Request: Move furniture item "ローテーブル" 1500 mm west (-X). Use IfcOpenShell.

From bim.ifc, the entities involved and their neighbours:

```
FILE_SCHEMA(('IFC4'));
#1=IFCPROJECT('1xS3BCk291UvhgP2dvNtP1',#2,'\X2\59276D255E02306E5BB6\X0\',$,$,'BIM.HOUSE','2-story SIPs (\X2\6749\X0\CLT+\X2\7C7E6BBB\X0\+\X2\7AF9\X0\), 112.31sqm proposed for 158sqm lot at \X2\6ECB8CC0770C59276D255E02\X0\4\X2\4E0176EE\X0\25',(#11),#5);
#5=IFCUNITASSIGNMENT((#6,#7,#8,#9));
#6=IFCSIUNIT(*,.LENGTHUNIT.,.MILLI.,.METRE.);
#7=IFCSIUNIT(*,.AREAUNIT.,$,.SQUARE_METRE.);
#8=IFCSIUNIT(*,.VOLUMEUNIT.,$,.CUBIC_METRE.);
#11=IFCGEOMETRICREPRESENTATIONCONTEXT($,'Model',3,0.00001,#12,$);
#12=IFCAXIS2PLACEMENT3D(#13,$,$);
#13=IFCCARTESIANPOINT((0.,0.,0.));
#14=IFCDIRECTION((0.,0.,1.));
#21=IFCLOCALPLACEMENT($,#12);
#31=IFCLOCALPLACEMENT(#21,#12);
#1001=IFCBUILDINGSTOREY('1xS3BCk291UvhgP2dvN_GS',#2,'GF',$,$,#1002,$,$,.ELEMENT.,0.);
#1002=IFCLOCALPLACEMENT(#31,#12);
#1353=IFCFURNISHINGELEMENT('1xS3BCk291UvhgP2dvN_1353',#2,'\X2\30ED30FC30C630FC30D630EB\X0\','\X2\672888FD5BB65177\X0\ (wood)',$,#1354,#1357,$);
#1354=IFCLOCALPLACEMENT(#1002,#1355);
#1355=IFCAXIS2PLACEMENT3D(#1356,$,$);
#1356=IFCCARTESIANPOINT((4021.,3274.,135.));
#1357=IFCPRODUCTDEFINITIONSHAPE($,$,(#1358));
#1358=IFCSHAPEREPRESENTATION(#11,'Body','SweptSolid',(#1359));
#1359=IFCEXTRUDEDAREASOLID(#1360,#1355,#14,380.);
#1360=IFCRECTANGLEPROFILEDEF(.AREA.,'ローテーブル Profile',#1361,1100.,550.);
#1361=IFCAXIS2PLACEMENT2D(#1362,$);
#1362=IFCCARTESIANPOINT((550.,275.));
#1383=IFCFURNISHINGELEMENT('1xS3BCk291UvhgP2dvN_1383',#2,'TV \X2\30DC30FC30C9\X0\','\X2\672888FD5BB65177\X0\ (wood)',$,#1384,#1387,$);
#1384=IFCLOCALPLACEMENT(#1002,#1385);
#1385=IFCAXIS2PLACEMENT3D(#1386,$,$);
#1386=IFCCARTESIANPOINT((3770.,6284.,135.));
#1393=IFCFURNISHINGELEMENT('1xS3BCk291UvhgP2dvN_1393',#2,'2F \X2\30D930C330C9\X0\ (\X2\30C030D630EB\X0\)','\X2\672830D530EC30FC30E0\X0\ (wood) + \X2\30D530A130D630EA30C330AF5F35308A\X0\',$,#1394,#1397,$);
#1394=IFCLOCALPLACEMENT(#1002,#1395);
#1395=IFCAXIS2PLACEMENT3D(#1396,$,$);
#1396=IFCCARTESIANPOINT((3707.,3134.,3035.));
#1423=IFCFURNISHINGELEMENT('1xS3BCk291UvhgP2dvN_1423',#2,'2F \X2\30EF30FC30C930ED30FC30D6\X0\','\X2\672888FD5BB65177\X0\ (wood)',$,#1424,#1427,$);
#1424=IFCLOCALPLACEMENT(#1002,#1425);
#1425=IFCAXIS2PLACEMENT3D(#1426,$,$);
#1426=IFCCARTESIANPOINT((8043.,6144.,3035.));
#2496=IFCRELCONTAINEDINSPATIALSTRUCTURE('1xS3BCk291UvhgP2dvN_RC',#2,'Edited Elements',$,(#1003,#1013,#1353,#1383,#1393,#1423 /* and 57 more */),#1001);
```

```python
import ifcopenshell
import ifcopenshell.api.geometry
import ifcopenshell.util.placement

model = ifcopenshell.open("bim.ifc")

item = model.by_id(1353)
matrix = ifcopenshell.util.placement.get_local_placement(item.ObjectPlacement)
matrix[0, 3] -= 1500.0
ifcopenshell.api.geometry.edit_object_placement(model, product=item, matrix=matrix, is_si=False)

print(ifcopenshell.util.placement.get_local_placement(item.ObjectPlacement).round(3) + 0.0)

model.write("bim-out.ifc")
```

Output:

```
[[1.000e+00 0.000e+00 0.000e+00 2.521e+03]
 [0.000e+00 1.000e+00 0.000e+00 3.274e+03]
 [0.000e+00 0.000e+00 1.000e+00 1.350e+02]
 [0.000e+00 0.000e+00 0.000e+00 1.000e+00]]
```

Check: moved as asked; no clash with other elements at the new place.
